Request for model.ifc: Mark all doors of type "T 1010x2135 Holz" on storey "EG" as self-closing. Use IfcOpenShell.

First a look at what the model holds.

```python
import ifcopenshell
import ifcopenshell.util.element

model = ifcopenshell.open("model.ifc")
print(model.schema)
storey = next(s for s in model.by_type("IfcBuildingStorey") if s.Name == "EG")
doors = [e for e in ifcopenshell.util.element.get_decomposition(storey) if e.is_a("IfcDoor")]
seen = {}
for e in doors:
    element_type = ifcopenshell.util.element.get_type(e)
    key = (element_type.Name if element_type != e and element_type else None, ifcopenshell.util.element.get_pset(e, "Pset_DoorCommon", "SelfClosing"))
    seen[key] = seen.get(key, 0) + 1
for (name, value), count in sorted(seen.items(), key=str):
    print(count, "x", name, "|", value)
```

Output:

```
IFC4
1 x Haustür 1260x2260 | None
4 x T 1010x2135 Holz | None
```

```python
import ifcopenshell
import ifcopenshell.api.pset
import ifcopenshell.util.element

model = ifcopenshell.open("model.ifc")

storey = next(s for s in model.by_type("IfcBuildingStorey") if s.Name == "EG")
doors = [e for e in ifcopenshell.util.element.get_decomposition(storey) if e.is_a("IfcDoor")]

count = 0
for e in doors:
    element_type = ifcopenshell.util.element.get_type(e)
    if element_type in (None, e) or element_type.Name != "T 1010x2135 Holz":
        continue
    # add_pset returns the element's existing set when there is one.
    pset = ifcopenshell.api.pset.add_pset(model, product=e, name="Pset_DoorCommon")
    ifcopenshell.api.pset.edit_pset(model, pset=pset, properties={"SelfClosing": True})
    count += 1

print(count, "doors updated")

model.write("model_rev.ifc")
```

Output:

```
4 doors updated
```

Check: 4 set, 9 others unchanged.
